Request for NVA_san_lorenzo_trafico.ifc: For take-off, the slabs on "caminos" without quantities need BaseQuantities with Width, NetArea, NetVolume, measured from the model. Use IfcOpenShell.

First a look at what the model holds.

```python
import ifcopenshell
import ifcopenshell.util.element
import ifcopenshell.util.unit

model = ifcopenshell.open("NVA_san_lorenzo_trafico.ifc")
print(model.schema)
for unit_type in ("LENGTHUNIT", "AREAUNIT", "VOLUMEUNIT"):
    print(unit_type, ifcopenshell.util.unit.calculate_unit_scale(model, unit_type))
storey = next(s for s in model.by_type("IfcBuildingStorey") if s.Name == "caminos")
slabs = [e for e in ifcopenshell.util.element.get_decomposition(storey) if e.is_a("IfcSlab")]
for e in sorted(slabs, key=lambda e: e.id()):
    print(e.id(), e.is_a(), e.Name, list(ifcopenshell.util.element.get_psets(e, qtos_only=True)), sep=" | ")
```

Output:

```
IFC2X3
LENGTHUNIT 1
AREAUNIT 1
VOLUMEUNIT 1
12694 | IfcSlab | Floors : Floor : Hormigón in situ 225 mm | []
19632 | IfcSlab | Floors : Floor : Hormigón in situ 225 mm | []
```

```python
import ifcopenshell
import ifcopenshell.api.pset
import ifcopenshell.geom
import ifcopenshell.util.element
import ifcopenshell.util.shape
import ifcopenshell.util.unit

model = ifcopenshell.open("NVA_san_lorenzo_trafico.ifc")
unit_scale = ifcopenshell.util.unit.calculate_unit_scale(model)
area_scale = ifcopenshell.util.unit.calculate_unit_scale(model, "AREAUNIT")
volume_scale = ifcopenshell.util.unit.calculate_unit_scale(model, "VOLUMEUNIT")
settings = ifcopenshell.geom.settings()

storey = next(s for s in model.by_type("IfcBuildingStorey") if s.Name == "caminos")
slabs = [e for e in ifcopenshell.util.element.get_decomposition(storey) if e.is_a("IfcSlab")]

for e in sorted(slabs, key=lambda e: e.id()):
    if ifcopenshell.util.element.get_psets(e, qtos_only=True, should_inherit=False):
        continue
    # Geometry comes back in metres, in the element's own axes.
    shape = ifcopenshell.geom.create_shape(settings, e)
    values = {
        "Width": ifcopenshell.util.shape.get_z(shape.geometry) / unit_scale,
        "NetArea": ifcopenshell.util.shape.get_footprint_area(shape.geometry) / area_scale,
        "NetVolume": ifcopenshell.util.shape.get_volume(shape.geometry) / volume_scale,
    }
    qto = ifcopenshell.api.pset.add_qto(model, product=e, name="BaseQuantities")
    ifcopenshell.api.pset.edit_qto(model, qto=qto, properties=values)
    print(e.id(), {k: round(v, 3) for k, v in values.items()})

model.write("NVA_san_lorenzo_trafico_edited.ifc")
```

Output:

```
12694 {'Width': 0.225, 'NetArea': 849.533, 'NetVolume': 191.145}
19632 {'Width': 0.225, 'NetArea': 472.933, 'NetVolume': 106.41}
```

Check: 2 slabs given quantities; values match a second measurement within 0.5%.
